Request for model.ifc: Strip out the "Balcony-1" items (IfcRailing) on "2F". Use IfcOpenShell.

First a look at what the model holds.

```python
import ifcopenshell
import ifcopenshell.util.element

model = ifcopenshell.open("model.ifc")
print(model.schema)
storey = next(s for s in model.by_type("IfcBuildingStorey") if s.Name == "2F")
railings = [e for e in ifcopenshell.util.element.get_decomposition(storey) if e.is_a("IfcRailing")]
seen = {}
for e in railings:
    element_type = ifcopenshell.util.element.get_type(e)
    name = element_type.Name if element_type not in (None, e) else None
    seen[name] = seen.get(name, 0) + 1
for name, count in sorted(seen.items(), key=str):
    print(count, "x", name)
```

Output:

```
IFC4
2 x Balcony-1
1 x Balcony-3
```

```python
import ifcopenshell
import ifcopenshell.api.root
import ifcopenshell.util.element

model = ifcopenshell.open("model.ifc")

storey = next(s for s in model.by_type("IfcBuildingStorey") if s.Name == "2F")
railings = [e for e in ifcopenshell.util.element.get_decomposition(storey) if e.is_a("IfcRailing")]
targets = [e for e in railings if (t := ifcopenshell.util.element.get_type(e)) not in (None, e) and t.Name == "Balcony-1"]

for e in targets:
    ifcopenshell.api.root.remove_product(model, product=e)
print(len(targets), "removed")

model.write("model_v2.ifc")
```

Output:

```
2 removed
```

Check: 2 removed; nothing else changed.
